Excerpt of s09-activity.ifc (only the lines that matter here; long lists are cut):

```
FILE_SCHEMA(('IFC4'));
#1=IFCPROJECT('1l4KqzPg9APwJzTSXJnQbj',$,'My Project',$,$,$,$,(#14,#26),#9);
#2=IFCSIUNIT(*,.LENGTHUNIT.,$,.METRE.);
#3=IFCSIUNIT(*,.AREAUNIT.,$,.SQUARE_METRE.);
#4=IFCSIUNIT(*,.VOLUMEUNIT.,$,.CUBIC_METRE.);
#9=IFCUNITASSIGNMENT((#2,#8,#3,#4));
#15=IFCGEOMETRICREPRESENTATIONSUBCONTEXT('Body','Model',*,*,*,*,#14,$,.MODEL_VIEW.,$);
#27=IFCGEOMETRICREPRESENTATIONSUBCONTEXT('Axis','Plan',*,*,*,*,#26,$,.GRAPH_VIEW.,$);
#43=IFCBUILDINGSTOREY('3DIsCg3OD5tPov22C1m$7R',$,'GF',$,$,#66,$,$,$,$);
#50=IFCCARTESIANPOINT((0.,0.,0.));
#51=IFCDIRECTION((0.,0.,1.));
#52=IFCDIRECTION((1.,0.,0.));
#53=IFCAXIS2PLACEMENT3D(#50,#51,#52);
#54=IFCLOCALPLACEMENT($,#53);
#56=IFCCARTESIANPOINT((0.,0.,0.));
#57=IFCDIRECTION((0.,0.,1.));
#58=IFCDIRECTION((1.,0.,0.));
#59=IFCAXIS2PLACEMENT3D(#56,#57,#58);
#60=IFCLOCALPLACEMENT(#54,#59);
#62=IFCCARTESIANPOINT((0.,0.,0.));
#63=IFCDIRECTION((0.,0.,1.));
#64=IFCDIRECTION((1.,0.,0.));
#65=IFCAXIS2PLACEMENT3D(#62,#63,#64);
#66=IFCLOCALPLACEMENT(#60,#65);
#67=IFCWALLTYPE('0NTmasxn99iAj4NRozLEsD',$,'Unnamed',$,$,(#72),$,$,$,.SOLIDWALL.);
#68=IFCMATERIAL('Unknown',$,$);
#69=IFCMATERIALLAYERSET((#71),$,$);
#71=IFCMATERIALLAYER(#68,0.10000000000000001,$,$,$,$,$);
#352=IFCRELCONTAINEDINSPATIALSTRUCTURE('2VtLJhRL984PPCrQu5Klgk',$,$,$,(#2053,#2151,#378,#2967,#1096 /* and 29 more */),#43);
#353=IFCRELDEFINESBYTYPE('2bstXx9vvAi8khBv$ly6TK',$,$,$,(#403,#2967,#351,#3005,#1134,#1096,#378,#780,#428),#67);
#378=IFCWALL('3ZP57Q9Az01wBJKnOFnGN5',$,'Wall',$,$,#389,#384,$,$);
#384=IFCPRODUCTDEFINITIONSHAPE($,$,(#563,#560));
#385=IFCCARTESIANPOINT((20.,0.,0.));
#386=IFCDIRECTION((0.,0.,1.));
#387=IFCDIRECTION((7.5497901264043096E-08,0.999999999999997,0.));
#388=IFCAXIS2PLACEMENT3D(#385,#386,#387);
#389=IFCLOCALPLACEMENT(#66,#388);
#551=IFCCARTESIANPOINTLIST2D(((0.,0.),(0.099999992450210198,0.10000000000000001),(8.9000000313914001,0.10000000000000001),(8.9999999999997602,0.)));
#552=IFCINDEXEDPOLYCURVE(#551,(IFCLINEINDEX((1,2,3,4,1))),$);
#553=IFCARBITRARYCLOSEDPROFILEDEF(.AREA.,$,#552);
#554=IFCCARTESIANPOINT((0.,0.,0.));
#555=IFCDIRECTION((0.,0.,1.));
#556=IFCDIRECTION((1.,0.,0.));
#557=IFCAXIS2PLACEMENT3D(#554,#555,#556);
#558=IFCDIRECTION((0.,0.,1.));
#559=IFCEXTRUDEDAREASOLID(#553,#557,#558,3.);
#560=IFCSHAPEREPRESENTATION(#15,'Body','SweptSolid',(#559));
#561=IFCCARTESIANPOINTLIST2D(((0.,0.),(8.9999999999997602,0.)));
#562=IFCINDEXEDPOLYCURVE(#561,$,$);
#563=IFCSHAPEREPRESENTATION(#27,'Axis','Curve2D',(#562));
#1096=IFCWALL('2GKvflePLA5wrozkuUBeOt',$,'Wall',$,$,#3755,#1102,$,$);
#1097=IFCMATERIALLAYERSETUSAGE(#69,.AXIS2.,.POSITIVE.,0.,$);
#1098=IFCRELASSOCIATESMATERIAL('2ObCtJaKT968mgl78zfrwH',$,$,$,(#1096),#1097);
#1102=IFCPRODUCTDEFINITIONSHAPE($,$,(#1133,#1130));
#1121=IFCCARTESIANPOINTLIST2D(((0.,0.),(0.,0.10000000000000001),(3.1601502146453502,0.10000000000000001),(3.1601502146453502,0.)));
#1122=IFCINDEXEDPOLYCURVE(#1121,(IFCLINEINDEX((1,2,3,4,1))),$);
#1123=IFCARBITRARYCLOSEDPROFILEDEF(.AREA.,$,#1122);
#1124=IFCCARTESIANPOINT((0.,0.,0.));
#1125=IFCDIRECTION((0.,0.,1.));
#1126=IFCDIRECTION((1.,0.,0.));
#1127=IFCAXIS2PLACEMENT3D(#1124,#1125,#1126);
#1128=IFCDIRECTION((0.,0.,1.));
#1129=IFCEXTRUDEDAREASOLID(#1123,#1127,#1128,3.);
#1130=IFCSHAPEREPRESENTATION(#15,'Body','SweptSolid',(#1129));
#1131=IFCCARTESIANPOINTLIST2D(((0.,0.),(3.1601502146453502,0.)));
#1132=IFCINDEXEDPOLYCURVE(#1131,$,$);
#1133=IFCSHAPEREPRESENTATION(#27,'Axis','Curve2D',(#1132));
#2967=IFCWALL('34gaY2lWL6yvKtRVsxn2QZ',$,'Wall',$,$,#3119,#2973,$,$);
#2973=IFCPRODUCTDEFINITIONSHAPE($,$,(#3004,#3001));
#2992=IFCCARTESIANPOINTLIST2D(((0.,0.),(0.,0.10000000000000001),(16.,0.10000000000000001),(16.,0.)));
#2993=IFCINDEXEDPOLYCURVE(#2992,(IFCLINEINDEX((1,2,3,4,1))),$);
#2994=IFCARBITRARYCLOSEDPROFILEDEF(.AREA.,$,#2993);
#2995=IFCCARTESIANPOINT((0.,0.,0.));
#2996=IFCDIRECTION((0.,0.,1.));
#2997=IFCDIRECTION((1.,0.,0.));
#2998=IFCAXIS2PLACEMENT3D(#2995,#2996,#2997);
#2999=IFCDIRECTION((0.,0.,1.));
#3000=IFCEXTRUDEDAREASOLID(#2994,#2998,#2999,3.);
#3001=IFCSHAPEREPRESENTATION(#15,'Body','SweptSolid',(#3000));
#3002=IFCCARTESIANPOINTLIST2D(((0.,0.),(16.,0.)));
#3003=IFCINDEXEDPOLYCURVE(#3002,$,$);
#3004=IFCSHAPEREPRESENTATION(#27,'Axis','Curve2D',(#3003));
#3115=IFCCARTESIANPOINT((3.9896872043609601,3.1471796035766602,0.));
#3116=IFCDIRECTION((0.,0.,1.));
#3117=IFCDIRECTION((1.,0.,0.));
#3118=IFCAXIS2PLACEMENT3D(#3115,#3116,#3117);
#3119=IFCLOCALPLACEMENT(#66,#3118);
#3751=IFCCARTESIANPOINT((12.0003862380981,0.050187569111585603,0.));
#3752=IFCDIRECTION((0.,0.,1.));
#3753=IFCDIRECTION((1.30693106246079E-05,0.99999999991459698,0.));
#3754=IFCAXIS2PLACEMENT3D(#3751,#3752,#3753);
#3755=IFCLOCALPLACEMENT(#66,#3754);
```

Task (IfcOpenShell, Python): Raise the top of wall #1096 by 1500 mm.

```python
import ifcopenshell
import ifcopenshell.geom
import ifcopenshell.util.representation
import ifcopenshell.util.shape
import ifcopenshell.util.unit

model = ifcopenshell.open("s09-activity.ifc")
unit_scale = ifcopenshell.util.unit.calculate_unit_scale(model)
settings = ifcopenshell.geom.settings()


def volume(element):
    """Net volume in cubic metres, openings subtracted."""
    shape = ifcopenshell.geom.create_shape(settings, element)
    return ifcopenshell.util.shape.get_volume(shape.geometry)


wall = model.by_guid("2GKvflePLA5wrozkuUBeOt")
before = volume(wall)

body = ifcopenshell.util.representation.get_representation(wall, "Model", "Body")
solid = body.Items[0]
old_height = solid.Depth
solid.Depth += 1.5 / unit_scale
after = volume(wall)

print(f"height {old_height:g} -> {solid.Depth:g}, volume {before:.3f} -> {after:.3f} m3")

model.write("s09-activity-out.ifc")
```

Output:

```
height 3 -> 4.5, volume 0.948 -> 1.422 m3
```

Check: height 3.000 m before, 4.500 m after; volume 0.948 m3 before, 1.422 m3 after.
